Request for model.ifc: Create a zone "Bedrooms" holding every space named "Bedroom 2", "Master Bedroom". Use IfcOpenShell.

First a look at what the model holds.

```python
import ifcopenshell

model = ifcopenshell.open("model.ifc")
print(model.schema)
seen = {}
for space in model.by_type("IfcSpace"):
    seen[space.LongName] = seen.get(space.LongName, 0) + 1
for name, count in sorted(seen.items(), key=str):
    print(count, "x", name)
print("zones:", [z.Name for z in model.by_type("IfcZone")][:20])
```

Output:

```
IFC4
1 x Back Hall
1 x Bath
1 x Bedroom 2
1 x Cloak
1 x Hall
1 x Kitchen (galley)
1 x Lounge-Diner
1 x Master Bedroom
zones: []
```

```python
import ifcopenshell
import ifcopenshell.api.group
import ifcopenshell.api.root

model = ifcopenshell.open("model.ifc")

names = {"Bedroom 2", "Master Bedroom"}
spaces = [s for s in model.by_type("IfcSpace") if s.LongName in names]

zone = ifcopenshell.api.root.create_entity(model, ifc_class="IfcZone", name="Bedrooms")
ifcopenshell.api.group.assign_group(model, products=spaces, group=zone)
print(len(spaces), "spaces in", zone.Name)

model.write("model_updated.ifc")
```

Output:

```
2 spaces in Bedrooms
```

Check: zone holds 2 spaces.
